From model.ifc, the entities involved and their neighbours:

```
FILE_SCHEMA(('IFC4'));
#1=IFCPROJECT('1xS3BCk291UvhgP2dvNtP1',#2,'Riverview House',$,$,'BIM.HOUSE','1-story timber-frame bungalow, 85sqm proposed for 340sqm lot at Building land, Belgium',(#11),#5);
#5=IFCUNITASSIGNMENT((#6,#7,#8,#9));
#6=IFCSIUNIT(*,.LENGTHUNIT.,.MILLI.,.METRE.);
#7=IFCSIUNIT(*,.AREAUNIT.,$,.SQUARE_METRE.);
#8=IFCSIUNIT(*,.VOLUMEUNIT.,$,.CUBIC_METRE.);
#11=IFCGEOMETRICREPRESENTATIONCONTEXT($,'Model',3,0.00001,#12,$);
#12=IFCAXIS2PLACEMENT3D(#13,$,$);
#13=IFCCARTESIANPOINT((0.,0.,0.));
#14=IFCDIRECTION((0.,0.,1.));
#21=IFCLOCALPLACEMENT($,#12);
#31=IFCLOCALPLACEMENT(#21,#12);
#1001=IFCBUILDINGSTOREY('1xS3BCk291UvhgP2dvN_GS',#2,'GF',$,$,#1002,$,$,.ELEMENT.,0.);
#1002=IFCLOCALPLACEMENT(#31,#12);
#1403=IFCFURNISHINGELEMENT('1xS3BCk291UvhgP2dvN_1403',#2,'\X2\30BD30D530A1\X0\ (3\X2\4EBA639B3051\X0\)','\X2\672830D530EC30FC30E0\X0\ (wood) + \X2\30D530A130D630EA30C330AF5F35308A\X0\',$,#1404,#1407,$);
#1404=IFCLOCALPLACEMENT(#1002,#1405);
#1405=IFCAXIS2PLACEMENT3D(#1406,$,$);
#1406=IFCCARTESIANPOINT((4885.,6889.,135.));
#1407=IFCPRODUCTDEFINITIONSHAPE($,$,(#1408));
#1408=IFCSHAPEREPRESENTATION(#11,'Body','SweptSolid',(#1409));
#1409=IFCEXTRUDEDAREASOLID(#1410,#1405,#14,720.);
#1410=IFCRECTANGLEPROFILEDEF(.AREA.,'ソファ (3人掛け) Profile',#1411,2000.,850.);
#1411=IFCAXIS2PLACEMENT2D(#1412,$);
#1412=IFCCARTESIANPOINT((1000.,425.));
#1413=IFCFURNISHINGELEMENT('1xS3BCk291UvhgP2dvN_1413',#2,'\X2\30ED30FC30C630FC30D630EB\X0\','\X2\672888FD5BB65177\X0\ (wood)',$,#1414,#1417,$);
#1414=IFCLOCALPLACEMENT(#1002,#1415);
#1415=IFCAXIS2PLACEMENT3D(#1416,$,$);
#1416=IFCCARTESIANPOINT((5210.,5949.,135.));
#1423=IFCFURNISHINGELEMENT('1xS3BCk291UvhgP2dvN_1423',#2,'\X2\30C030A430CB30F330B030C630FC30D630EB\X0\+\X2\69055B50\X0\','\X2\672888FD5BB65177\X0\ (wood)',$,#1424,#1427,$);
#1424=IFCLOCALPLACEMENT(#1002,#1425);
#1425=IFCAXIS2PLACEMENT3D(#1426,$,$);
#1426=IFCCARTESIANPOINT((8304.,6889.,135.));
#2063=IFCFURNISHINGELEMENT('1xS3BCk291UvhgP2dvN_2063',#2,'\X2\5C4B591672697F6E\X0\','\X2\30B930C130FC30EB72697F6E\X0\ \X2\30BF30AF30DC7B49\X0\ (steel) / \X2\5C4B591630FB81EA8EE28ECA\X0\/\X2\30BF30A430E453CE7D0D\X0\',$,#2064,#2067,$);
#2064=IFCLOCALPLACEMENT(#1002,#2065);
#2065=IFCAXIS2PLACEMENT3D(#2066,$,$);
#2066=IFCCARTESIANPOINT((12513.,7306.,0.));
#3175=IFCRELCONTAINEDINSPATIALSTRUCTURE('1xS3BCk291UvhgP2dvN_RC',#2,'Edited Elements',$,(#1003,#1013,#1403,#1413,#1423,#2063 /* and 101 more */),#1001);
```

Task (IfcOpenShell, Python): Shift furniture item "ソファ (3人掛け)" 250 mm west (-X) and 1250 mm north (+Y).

```python
import ifcopenshell
import ifcopenshell.api.geometry
import ifcopenshell.util.placement
import ifcopenshell.util.unit

model = ifcopenshell.open("model.ifc")
unit_scale = ifcopenshell.util.unit.calculate_unit_scale(model)

item = model.by_id(1403)
matrix = ifcopenshell.util.placement.get_local_placement(item.ObjectPlacement)
matrix[0, 3] -= 0.25 / unit_scale
matrix[1, 3] += 1.25 / unit_scale
ifcopenshell.api.geometry.edit_object_placement(model, product=item, matrix=matrix, is_si=False)

print(ifcopenshell.util.placement.get_local_placement(item.ObjectPlacement).round(3) + 0.0)

model.write("model_updated.ifc")
```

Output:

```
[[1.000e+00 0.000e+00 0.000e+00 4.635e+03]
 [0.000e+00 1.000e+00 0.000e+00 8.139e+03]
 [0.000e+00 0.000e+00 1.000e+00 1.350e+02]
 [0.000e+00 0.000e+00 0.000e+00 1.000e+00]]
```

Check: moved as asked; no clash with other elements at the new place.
